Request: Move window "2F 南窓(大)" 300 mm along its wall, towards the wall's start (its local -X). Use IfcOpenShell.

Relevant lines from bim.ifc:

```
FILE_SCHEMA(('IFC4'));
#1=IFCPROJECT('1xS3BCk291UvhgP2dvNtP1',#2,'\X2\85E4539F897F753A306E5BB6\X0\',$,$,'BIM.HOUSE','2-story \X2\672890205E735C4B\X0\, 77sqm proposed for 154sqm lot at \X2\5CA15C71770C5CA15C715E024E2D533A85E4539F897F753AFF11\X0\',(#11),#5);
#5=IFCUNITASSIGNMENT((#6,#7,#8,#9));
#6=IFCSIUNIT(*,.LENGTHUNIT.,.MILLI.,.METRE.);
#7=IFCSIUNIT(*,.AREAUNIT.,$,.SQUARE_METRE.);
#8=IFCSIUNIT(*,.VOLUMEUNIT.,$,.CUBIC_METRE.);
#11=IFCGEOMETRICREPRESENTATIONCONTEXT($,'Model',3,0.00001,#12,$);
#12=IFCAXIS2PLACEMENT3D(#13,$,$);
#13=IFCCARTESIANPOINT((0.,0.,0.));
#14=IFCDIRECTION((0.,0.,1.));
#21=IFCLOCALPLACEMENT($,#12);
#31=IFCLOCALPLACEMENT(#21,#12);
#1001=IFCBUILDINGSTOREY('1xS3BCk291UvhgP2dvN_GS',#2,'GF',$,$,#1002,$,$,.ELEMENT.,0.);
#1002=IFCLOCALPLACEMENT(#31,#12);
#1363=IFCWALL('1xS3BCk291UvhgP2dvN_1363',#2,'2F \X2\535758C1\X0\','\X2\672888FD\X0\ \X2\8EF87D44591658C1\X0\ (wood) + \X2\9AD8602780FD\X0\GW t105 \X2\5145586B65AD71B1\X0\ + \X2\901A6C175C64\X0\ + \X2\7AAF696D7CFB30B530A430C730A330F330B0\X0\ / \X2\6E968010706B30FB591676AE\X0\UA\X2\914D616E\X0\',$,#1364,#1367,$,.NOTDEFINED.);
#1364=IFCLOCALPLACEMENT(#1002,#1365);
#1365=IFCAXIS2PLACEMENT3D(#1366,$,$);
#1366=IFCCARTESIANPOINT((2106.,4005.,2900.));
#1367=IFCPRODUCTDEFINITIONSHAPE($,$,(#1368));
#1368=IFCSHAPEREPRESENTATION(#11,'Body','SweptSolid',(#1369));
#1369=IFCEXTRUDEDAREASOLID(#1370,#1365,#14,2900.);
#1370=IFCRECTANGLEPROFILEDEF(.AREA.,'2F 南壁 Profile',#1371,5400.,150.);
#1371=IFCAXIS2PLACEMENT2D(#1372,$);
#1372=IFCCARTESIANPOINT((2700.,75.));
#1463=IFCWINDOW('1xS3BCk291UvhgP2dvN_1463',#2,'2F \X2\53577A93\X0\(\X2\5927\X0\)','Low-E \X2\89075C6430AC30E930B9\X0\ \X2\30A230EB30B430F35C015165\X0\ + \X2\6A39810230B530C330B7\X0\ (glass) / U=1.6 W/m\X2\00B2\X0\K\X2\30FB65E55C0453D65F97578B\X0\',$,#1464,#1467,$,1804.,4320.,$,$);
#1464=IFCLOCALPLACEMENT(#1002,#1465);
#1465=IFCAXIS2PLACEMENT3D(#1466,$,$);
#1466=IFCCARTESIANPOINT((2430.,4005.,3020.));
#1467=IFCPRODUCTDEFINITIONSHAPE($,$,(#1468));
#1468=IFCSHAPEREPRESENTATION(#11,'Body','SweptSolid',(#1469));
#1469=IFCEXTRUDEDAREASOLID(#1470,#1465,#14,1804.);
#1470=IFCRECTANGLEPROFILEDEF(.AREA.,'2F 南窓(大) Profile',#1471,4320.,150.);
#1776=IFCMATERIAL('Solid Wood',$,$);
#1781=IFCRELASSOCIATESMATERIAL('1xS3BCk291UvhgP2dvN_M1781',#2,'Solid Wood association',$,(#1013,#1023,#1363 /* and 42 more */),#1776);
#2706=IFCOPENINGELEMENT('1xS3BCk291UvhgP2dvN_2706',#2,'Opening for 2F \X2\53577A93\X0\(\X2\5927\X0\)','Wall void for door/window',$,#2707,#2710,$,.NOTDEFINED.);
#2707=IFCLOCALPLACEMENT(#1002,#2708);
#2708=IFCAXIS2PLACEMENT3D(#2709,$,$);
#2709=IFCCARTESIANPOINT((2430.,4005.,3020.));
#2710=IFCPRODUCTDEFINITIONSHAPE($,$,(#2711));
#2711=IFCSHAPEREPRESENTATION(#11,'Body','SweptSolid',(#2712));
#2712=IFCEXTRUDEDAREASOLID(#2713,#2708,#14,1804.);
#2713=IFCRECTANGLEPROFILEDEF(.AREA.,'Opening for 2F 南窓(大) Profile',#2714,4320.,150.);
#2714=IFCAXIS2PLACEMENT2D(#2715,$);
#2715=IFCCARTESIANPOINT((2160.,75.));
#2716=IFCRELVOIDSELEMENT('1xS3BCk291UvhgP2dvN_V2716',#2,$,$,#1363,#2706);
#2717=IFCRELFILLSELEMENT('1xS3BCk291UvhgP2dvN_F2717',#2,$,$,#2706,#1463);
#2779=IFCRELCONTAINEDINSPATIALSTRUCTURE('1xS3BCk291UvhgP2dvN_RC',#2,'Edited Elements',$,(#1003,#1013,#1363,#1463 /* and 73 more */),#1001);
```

```python
import ifcopenshell
import ifcopenshell.api.geometry
import ifcopenshell.util.placement
import ifcopenshell.util.unit

model = ifcopenshell.open("bim.ifc")
unit_scale = ifcopenshell.util.unit.calculate_unit_scale(model)

window = model.by_guid("1xS3BCk291UvhgP2dvN_1463")
opening = window.FillsVoids[0].RelatingOpeningElement
wall = opening.VoidsElements[0].RelatingBuildingElement

wall_matrix = ifcopenshell.util.placement.get_local_placement(wall.ObjectPlacement)
shift = wall_matrix[:3, 0] * -0.3 / unit_scale
before = ifcopenshell.util.placement.get_local_placement(window.ObjectPlacement)[:3, 3].copy()

# The window is not placed relative to its opening, so move both.
for product in (opening, window):
    matrix = ifcopenshell.util.placement.get_local_placement(product.ObjectPlacement)
    matrix[:3, 3] += shift
    ifcopenshell.api.geometry.edit_object_placement(model, product=product, matrix=matrix, is_si=False)

after = ifcopenshell.util.placement.get_local_placement(window.ObjectPlacement)[:3, 3]
print("window moved by", (after - before).round(3) + 0.0)

model.write("bim_edited.ifc")
```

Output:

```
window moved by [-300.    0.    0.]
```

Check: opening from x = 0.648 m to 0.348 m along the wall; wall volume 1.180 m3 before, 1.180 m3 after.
